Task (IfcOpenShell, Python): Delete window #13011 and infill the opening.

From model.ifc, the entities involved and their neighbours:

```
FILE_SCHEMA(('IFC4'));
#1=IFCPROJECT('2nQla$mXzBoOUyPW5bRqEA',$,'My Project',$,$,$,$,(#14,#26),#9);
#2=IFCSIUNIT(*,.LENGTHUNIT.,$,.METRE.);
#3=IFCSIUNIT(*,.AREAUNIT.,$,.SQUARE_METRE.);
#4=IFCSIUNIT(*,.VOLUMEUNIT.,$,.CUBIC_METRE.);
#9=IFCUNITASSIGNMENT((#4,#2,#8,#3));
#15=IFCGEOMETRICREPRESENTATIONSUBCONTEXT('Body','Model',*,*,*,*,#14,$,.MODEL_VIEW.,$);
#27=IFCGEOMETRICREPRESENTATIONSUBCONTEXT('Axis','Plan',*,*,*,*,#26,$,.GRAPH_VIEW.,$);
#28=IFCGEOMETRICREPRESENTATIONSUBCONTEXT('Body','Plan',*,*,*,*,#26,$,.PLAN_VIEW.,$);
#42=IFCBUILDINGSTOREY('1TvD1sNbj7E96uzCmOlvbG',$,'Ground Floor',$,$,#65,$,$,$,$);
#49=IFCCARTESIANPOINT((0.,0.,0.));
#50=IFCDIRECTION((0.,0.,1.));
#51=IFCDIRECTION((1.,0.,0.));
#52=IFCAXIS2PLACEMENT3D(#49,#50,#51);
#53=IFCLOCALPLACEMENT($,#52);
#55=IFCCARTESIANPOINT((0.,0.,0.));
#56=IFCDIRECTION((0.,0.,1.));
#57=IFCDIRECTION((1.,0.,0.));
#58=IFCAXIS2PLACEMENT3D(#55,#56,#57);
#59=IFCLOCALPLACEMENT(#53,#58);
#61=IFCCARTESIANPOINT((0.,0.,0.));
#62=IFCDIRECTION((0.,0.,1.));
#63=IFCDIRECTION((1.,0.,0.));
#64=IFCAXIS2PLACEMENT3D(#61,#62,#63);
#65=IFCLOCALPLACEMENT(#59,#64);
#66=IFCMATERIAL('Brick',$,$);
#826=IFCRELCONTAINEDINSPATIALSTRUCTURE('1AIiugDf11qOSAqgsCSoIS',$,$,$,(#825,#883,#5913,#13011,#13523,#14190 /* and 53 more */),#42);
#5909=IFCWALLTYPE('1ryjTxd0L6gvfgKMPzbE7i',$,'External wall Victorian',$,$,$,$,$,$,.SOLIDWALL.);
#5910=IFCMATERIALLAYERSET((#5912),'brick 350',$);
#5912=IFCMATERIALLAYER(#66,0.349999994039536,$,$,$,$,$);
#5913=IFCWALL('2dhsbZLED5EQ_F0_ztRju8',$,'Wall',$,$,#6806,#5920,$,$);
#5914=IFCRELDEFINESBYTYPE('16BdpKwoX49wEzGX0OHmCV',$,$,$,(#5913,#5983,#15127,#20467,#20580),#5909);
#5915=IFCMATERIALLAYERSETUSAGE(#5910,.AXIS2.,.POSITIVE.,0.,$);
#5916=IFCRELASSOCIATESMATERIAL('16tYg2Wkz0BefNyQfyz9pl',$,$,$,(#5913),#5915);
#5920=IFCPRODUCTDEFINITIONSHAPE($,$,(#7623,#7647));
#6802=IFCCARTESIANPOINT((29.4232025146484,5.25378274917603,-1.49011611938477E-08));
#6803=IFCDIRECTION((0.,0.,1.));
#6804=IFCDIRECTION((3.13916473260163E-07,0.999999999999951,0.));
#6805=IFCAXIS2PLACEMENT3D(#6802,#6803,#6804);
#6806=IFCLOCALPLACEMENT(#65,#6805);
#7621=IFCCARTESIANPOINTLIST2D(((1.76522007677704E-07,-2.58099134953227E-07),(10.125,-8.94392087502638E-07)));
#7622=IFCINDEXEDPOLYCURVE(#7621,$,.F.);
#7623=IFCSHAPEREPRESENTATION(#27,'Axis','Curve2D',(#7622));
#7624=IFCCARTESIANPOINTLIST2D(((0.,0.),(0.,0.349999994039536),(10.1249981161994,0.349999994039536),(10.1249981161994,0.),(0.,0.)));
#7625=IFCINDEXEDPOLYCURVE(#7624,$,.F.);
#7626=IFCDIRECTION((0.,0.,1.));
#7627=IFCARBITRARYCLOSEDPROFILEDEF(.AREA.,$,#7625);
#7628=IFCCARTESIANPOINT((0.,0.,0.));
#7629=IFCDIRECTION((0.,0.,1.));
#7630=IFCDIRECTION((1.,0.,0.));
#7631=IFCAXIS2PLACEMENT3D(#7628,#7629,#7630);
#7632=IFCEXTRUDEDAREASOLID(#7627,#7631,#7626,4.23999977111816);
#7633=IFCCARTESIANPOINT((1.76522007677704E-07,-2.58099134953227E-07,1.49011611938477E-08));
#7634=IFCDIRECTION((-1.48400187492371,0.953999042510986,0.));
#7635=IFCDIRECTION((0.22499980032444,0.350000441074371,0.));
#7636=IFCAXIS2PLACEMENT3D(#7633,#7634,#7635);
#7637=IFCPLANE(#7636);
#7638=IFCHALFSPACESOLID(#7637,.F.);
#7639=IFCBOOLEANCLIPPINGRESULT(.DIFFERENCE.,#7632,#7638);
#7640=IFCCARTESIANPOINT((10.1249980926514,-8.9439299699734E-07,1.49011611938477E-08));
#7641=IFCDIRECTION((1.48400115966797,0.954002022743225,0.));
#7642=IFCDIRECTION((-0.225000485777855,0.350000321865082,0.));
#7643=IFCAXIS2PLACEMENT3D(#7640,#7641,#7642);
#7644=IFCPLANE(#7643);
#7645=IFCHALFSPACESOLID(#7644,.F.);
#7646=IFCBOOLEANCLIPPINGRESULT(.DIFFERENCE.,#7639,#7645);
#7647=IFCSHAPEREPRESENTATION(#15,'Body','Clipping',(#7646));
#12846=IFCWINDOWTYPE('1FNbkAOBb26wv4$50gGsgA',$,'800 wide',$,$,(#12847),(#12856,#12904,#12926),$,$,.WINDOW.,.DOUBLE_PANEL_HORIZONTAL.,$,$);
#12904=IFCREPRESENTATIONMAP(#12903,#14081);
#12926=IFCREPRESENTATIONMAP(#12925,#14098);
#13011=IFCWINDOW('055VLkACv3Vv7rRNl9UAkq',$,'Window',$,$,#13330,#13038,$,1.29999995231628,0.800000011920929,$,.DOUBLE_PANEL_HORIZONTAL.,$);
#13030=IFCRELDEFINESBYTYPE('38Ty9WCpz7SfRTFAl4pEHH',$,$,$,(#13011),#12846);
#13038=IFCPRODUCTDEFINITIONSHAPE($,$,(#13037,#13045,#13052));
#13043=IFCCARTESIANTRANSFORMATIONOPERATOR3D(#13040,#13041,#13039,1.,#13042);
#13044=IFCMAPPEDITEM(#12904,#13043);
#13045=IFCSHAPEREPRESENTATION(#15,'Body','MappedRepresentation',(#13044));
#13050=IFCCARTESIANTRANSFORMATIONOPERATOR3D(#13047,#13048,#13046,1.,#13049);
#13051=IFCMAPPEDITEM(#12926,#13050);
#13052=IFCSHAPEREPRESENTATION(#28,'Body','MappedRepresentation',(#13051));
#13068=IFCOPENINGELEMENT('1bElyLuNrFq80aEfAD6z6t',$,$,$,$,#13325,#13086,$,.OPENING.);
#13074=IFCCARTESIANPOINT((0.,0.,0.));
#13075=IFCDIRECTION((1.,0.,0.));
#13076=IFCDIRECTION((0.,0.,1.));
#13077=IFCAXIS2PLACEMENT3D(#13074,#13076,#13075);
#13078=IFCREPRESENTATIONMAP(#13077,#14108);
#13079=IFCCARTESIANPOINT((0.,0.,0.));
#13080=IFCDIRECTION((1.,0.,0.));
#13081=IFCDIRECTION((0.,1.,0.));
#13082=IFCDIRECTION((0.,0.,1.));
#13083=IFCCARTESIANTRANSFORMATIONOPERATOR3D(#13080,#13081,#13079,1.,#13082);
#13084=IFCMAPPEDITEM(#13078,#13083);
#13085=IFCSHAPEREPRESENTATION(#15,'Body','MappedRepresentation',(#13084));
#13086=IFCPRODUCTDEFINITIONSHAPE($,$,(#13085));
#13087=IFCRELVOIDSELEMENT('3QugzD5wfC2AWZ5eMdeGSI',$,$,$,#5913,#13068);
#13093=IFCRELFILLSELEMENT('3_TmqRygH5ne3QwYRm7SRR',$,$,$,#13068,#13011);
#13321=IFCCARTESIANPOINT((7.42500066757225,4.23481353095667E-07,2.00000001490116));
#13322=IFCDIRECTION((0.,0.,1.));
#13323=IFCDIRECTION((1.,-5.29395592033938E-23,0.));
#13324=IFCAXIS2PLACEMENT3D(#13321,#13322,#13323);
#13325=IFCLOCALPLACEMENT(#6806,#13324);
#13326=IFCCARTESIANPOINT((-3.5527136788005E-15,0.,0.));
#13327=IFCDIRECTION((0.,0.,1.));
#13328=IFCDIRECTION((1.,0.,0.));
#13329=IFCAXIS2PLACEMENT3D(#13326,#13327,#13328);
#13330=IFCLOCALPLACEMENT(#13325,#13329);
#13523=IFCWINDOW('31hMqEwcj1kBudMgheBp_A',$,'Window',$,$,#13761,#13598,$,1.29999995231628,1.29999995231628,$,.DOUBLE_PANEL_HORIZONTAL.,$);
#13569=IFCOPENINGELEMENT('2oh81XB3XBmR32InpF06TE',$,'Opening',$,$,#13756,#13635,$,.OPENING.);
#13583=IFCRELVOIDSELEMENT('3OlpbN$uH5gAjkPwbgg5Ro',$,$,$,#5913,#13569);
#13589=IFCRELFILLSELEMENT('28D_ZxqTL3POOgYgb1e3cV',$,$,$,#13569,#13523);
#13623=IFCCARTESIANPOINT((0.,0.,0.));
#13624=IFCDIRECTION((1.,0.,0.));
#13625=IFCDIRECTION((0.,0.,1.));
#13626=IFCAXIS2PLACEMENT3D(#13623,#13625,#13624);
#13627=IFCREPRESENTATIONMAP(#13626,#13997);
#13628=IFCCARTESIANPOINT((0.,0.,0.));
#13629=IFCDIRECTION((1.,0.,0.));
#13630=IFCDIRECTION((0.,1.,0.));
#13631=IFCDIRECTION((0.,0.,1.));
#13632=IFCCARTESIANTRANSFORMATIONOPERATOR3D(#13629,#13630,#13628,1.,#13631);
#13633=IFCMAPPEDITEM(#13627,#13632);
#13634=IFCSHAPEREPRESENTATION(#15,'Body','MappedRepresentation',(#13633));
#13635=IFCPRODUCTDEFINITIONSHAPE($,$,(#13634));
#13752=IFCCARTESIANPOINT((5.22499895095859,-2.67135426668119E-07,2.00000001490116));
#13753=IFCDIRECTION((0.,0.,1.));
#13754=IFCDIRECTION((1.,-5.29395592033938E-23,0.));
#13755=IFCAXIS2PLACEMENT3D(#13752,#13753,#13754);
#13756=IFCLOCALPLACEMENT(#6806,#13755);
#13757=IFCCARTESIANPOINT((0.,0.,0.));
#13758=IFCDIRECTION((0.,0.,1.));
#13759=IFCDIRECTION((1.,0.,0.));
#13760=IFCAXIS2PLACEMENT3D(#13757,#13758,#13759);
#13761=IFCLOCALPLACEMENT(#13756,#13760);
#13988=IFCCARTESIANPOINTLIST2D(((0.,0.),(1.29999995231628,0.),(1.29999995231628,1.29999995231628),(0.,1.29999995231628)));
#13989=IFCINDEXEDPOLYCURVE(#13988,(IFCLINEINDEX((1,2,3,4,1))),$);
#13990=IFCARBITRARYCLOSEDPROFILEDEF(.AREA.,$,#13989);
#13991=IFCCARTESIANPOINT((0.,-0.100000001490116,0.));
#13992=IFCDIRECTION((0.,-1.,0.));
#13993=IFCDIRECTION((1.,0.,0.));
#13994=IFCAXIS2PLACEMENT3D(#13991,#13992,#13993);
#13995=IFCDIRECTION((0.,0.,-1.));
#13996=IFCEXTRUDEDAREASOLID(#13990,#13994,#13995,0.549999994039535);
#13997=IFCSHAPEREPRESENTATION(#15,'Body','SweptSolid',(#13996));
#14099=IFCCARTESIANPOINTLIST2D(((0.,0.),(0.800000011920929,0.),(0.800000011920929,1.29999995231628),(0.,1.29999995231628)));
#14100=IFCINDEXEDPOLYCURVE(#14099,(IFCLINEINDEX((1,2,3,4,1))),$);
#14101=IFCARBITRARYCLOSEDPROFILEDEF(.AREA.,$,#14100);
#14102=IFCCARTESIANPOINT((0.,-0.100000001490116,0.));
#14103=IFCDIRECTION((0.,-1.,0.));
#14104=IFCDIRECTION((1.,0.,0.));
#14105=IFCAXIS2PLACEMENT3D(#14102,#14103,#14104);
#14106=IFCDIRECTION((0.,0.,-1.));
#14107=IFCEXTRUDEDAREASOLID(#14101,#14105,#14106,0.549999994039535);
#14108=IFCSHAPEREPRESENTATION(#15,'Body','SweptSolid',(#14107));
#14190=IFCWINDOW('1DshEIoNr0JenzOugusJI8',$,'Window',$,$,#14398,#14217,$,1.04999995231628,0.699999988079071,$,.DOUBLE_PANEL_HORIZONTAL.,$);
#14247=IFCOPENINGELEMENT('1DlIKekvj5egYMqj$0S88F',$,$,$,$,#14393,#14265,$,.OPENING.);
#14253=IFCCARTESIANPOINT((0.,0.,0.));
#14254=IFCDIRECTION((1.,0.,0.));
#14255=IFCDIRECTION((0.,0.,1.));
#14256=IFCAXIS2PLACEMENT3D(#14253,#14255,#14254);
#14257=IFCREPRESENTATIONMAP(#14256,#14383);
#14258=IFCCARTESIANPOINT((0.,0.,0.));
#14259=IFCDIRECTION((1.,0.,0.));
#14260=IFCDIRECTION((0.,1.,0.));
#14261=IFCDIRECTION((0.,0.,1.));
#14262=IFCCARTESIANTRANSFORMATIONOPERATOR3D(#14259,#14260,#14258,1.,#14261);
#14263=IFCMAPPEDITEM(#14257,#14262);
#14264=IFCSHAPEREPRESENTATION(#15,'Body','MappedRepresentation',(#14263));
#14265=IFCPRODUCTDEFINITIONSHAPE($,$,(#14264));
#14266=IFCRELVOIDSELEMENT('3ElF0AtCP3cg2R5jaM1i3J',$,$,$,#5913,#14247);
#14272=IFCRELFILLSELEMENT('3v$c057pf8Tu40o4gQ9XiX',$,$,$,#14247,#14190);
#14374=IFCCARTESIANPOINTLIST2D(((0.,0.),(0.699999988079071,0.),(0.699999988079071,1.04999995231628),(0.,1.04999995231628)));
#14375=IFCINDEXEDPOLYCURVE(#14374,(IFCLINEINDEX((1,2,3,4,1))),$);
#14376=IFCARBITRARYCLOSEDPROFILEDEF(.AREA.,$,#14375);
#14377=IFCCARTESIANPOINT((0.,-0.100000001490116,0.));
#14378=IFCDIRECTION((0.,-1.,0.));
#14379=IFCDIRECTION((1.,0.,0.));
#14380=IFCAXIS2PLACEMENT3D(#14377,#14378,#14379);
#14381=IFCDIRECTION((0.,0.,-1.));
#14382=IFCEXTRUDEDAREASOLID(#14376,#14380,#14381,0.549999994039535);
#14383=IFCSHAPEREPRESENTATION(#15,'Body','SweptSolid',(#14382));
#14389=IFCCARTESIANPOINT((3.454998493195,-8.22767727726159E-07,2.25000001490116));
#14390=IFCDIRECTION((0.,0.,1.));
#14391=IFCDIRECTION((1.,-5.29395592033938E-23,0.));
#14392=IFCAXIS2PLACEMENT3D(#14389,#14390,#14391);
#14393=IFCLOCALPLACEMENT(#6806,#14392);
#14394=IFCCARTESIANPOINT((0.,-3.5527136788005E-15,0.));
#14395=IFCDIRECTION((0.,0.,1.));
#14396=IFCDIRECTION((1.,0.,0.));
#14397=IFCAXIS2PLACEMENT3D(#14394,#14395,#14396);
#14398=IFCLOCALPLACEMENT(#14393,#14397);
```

```python
import ifcopenshell
import ifcopenshell.api.feature
import ifcopenshell.api.root
import ifcopenshell.geom
import ifcopenshell.util.shape

model = ifcopenshell.open("model.ifc")
settings = ifcopenshell.geom.settings()


def volume(element):
    """Net volume in cubic metres, openings subtracted."""
    shape = ifcopenshell.geom.create_shape(settings, element)
    return ifcopenshell.util.shape.get_volume(shape.geometry)


window = model.by_id(13011)
opening = window.FillsVoids[0].RelatingOpeningElement
wall = opening.VoidsElements[0].RelatingBuildingElement
before = volume(wall)

ifcopenshell.api.root.remove_product(model, product=window)
ifcopenshell.api.feature.remove_feature(model, feature=opening)

after = volume(wall)

print(f"wall volume {before:.3f} -> {after:.3f} m3")

model.write("model-out.ifc")
```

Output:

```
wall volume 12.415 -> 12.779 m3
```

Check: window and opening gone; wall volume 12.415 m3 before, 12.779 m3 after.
